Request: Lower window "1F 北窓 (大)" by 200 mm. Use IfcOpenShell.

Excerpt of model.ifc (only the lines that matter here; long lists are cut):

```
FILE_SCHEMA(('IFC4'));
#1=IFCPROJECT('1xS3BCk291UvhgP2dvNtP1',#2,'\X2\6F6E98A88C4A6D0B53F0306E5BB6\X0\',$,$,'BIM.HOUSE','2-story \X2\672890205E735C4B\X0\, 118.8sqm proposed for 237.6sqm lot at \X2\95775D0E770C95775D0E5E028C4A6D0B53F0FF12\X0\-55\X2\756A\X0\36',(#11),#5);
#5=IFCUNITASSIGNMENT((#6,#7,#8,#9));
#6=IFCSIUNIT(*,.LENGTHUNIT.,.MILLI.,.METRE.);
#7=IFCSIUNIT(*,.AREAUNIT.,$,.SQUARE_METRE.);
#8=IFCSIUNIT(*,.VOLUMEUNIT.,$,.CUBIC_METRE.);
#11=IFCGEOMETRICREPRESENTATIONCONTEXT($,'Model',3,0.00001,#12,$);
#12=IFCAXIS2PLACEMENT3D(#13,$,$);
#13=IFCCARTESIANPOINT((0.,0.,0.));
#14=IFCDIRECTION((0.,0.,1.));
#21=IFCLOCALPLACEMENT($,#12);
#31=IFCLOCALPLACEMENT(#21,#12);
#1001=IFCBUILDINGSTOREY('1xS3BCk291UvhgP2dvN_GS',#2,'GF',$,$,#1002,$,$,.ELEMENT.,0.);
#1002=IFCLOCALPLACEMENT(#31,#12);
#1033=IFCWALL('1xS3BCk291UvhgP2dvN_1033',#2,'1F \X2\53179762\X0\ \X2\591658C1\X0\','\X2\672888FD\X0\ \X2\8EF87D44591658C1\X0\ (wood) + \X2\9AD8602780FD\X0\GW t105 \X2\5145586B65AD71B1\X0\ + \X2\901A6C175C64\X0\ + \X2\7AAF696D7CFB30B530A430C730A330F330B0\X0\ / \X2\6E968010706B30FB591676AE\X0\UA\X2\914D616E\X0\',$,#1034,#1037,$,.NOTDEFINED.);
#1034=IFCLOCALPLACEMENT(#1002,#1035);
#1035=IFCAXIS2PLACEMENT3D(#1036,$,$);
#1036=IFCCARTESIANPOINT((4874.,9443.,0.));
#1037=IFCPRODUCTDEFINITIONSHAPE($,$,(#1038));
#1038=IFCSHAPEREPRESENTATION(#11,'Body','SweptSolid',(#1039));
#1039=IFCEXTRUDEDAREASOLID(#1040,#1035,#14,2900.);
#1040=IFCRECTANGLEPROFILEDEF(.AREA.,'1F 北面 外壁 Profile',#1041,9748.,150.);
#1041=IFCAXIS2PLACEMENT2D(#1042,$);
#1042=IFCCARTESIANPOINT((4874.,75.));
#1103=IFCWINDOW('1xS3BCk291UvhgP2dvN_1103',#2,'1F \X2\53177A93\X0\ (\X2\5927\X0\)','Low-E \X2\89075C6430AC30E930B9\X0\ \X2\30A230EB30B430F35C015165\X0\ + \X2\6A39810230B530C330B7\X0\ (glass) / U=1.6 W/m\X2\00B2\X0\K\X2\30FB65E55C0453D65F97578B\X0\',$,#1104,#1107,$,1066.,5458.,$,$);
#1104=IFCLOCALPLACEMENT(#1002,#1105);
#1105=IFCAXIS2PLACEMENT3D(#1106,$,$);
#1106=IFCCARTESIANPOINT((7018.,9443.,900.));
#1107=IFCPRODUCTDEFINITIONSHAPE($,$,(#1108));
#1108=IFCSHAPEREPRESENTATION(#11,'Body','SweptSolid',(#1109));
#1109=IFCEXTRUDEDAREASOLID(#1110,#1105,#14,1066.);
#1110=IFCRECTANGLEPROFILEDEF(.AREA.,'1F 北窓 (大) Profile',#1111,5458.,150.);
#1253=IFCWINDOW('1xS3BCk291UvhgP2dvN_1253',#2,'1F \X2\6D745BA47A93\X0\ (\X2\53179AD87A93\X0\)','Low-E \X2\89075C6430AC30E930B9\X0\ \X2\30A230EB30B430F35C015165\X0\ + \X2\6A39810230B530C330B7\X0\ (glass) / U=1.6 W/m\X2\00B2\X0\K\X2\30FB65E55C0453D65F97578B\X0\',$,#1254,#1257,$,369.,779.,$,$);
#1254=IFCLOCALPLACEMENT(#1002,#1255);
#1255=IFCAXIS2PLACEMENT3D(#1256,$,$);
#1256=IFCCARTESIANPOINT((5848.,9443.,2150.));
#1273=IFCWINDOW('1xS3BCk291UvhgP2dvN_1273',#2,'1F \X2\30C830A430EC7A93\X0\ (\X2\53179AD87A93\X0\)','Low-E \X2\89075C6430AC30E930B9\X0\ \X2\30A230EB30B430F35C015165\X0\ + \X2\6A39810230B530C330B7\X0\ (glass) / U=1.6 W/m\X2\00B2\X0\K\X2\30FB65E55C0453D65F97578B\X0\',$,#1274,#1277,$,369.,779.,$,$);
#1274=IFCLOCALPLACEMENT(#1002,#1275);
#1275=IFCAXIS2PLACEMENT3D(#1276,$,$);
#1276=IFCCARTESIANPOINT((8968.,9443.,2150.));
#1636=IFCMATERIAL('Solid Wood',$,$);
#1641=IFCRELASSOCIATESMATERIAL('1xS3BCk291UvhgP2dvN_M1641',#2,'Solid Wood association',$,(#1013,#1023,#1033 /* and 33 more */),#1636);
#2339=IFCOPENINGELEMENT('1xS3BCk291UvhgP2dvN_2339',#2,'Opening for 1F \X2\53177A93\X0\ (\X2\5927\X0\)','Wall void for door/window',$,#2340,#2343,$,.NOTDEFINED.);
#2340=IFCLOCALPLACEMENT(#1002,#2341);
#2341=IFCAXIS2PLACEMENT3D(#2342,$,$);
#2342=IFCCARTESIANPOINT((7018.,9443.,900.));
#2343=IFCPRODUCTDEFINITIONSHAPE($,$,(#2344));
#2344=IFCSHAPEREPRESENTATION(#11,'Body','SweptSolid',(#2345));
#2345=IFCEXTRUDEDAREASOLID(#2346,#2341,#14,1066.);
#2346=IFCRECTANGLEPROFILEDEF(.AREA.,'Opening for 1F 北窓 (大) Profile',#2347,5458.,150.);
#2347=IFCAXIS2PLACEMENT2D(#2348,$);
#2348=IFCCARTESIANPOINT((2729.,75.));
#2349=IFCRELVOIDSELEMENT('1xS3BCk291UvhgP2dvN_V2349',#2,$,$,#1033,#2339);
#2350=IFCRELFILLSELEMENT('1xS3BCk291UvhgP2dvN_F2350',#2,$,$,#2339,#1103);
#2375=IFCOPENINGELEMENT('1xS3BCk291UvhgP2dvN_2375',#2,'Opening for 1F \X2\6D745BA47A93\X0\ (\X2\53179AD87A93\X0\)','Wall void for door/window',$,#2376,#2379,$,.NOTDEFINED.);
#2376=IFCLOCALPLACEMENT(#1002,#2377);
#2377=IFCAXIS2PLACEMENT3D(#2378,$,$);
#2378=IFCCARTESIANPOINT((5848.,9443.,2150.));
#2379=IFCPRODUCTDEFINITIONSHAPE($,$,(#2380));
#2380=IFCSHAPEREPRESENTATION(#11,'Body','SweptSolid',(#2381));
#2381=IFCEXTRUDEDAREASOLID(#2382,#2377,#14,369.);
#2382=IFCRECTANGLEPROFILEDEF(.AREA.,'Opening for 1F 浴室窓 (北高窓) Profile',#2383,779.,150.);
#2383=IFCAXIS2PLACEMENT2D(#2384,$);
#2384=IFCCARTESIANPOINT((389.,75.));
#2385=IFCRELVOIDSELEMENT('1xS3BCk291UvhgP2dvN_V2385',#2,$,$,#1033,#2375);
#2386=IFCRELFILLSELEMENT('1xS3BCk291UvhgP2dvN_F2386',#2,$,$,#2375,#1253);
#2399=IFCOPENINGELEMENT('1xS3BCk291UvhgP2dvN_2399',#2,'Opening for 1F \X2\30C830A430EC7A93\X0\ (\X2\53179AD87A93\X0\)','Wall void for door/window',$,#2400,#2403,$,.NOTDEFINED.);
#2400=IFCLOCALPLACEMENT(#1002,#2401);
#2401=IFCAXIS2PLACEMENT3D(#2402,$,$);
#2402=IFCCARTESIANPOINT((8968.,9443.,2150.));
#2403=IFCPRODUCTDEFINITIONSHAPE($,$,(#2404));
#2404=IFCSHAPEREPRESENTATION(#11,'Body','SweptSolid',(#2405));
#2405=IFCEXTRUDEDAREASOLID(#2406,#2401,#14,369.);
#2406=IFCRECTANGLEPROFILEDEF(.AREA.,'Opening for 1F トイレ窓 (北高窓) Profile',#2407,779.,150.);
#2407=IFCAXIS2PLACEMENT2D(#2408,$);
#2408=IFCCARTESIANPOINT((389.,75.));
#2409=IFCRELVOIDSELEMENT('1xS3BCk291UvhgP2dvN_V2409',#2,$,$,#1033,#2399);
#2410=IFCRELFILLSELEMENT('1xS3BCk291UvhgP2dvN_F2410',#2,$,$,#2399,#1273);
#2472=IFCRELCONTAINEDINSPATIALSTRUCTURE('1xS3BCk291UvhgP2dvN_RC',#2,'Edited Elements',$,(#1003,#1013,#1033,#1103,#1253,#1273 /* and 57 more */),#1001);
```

```python
import numpy as np
import ifcopenshell
import ifcopenshell.api.geometry
import ifcopenshell.util.placement
import ifcopenshell.util.unit

model = ifcopenshell.open("model.ifc")
unit_scale = ifcopenshell.util.unit.calculate_unit_scale(model)

window = model.by_id(1103)
opening = window.FillsVoids[0].RelatingOpeningElement
dz = -200.0

shift = np.array([0.0, 0.0, dz])
# The window is not placed relative to its opening, so move both.
for product in (opening, window):
    matrix = ifcopenshell.util.placement.get_local_placement(product.ObjectPlacement)
    matrix[:3, 3] += shift
    ifcopenshell.api.geometry.edit_object_placement(model, product=product, matrix=matrix, is_si=False)

print(f"moved by {dz * unit_scale:+.3f} m")

model.write("model_updated.ifc")
```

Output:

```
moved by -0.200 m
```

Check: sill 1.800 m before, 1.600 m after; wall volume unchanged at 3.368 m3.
